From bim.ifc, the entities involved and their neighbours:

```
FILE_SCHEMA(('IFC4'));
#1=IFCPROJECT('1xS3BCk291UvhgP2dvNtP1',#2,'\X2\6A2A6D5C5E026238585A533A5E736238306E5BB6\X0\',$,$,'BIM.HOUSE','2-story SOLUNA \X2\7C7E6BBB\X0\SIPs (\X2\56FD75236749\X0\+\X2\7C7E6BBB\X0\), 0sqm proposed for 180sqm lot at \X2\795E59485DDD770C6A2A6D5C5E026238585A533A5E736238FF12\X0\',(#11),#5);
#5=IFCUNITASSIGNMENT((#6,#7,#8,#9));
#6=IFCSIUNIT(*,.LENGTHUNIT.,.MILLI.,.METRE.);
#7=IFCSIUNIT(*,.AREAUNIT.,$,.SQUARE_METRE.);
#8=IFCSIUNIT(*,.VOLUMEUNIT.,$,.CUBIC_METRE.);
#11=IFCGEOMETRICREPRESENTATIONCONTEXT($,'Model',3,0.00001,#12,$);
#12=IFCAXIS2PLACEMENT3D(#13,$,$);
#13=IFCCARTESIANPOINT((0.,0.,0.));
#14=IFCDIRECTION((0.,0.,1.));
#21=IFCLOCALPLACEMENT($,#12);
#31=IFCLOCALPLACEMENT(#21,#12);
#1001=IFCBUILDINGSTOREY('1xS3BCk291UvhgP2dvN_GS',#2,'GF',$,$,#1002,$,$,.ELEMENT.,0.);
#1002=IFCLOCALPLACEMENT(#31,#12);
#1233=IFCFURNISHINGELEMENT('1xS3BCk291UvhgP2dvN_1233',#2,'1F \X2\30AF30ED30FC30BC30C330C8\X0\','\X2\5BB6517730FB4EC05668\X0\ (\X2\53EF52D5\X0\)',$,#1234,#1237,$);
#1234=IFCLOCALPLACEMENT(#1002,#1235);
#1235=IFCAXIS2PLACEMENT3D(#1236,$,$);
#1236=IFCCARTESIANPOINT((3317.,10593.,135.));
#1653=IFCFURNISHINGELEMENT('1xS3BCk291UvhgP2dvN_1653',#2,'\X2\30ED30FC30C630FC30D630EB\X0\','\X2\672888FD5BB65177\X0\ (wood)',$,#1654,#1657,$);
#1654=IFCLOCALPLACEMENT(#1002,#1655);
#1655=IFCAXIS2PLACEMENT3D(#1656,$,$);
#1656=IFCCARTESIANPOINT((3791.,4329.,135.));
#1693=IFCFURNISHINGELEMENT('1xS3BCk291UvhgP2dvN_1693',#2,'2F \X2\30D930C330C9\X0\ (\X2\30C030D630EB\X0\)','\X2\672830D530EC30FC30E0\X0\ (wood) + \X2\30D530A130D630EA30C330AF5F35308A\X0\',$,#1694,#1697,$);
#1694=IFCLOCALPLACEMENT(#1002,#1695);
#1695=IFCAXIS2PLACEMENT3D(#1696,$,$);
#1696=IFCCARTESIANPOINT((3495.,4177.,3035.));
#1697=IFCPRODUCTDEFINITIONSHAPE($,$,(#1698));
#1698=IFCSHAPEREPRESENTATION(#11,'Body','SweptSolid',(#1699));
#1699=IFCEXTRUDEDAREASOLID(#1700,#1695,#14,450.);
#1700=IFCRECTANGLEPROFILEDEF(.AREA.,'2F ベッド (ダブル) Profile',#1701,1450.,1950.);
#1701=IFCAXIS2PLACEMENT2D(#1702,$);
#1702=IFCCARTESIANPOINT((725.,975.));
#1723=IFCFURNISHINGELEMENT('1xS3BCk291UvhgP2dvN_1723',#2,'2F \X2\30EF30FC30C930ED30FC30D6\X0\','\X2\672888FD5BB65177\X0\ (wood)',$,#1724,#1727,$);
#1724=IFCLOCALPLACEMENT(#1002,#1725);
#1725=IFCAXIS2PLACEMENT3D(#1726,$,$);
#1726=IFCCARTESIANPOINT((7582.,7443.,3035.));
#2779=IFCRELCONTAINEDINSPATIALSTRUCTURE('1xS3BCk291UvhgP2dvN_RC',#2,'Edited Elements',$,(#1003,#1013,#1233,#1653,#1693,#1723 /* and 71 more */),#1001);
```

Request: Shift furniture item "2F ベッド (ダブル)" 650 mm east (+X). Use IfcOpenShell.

```python
import ifcopenshell
import ifcopenshell.api.geometry
import ifcopenshell.util.placement

model = ifcopenshell.open("bim.ifc")

item = model.by_guid("1xS3BCk291UvhgP2dvN_1693")
matrix = ifcopenshell.util.placement.get_local_placement(item.ObjectPlacement)
matrix[0, 3] += 650.0
ifcopenshell.api.geometry.edit_object_placement(model, product=item, matrix=matrix, is_si=False)

print(ifcopenshell.util.placement.get_local_placement(item.ObjectPlacement).round(3) + 0.0)

model.write("bim_v2.ifc")
```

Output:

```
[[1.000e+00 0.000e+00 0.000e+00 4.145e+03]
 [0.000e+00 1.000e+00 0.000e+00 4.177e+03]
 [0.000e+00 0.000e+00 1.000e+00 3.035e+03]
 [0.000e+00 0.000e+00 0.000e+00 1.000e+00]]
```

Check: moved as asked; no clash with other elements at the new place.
